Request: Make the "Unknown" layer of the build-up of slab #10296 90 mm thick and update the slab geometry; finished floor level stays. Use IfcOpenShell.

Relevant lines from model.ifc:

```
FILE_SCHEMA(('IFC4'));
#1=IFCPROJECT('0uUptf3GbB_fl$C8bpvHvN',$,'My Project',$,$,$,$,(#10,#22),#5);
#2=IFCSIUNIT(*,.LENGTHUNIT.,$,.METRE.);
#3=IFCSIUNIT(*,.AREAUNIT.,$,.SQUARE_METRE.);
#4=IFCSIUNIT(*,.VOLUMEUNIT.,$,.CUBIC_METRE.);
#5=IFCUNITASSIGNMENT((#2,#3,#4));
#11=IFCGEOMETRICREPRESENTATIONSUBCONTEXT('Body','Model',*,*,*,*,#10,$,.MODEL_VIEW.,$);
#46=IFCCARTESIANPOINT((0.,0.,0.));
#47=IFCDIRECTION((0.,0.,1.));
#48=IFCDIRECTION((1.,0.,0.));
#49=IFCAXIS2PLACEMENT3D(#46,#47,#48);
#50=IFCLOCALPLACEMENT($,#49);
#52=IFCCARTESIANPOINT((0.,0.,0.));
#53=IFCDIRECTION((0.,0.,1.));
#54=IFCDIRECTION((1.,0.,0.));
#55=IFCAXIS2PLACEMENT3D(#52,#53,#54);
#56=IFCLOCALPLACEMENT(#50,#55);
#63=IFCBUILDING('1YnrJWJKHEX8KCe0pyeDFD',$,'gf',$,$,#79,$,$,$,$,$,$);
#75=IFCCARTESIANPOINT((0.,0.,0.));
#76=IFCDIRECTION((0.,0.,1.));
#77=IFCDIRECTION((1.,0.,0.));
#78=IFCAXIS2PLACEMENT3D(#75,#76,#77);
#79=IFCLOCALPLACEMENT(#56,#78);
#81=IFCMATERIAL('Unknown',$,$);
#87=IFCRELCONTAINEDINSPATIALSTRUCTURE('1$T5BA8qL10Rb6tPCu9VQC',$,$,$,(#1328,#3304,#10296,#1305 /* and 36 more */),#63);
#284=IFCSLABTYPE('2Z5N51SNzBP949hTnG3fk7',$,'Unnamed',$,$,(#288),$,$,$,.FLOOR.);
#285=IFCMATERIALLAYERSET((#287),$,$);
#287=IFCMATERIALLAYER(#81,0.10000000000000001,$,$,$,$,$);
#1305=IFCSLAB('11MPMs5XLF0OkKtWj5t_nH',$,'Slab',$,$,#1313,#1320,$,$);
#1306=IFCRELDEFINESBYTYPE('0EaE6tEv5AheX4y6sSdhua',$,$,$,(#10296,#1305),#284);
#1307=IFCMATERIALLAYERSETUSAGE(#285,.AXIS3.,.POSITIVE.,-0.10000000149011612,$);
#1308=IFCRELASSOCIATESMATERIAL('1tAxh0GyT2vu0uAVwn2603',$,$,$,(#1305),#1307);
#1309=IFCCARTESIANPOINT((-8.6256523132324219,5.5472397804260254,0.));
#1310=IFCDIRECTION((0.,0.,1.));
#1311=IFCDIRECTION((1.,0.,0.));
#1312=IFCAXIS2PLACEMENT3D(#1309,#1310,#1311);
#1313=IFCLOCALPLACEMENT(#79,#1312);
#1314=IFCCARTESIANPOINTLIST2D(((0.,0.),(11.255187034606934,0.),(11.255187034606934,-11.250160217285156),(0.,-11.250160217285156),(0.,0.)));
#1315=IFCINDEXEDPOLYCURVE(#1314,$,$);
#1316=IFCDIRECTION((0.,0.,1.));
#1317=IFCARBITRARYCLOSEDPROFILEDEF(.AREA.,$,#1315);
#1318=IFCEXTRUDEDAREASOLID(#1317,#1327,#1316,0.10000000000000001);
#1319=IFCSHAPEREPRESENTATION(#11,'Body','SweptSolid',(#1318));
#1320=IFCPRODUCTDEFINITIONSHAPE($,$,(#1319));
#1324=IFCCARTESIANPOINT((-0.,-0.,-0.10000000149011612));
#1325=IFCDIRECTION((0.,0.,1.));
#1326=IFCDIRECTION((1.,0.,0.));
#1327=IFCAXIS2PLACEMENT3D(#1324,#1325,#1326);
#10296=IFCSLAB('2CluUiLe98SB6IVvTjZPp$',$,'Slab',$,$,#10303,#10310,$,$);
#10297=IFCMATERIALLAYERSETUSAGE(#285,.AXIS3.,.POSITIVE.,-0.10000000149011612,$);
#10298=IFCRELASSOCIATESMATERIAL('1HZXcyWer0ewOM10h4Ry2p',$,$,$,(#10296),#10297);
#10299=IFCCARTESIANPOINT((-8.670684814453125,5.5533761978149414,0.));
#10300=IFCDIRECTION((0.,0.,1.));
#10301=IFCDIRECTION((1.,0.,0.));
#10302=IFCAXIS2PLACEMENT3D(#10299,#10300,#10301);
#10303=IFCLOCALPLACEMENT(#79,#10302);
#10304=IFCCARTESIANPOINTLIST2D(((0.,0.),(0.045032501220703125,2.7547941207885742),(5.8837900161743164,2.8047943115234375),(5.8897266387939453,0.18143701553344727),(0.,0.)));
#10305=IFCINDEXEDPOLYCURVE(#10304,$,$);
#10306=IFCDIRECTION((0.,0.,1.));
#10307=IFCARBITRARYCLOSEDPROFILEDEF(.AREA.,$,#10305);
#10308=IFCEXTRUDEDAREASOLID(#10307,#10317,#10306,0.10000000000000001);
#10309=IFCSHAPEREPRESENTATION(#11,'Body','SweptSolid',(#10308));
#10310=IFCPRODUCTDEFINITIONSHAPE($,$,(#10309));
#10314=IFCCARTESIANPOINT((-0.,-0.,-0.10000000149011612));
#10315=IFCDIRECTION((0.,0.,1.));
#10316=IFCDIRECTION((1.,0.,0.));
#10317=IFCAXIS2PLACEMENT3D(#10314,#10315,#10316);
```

```python
import ifcopenshell
import ifcopenshell.util.element
import ifcopenshell.util.representation
import ifcopenshell.util.unit

model = ifcopenshell.open("model.ifc")
unit_scale = ifcopenshell.util.unit.calculate_unit_scale(model)

layer_set = model.by_id(285)
layer = next(l for l in layer_set.MaterialLayers if l.Material and l.Material.Name == "Unknown")
change = 0.09 / unit_scale - layer.LayerThickness
layer.LayerThickness += change

# The layer set is shared, so every slab that uses it gets the new thickness.
slabs = [e for e in ifcopenshell.util.element.get_elements_by_material(model, layer_set) if e.is_a("IfcSlab")]
for slab in sorted(slabs, key=lambda e: e.id()):
    body = ifcopenshell.util.representation.get_representation(slab, "Model", "Body")
    solid = body.Items[0]
    old_depth = solid.Depth
    solid.Depth += change
    # Extruded upwards: lower the start of the extrusion so the top stays.
    x, y, z = solid.Position.Location.Coordinates
    solid.Position.Location = model.createIfcCartesianPoint((x, y, z - change))
    print(slab.id(), f"{old_depth:g} -> {solid.Depth:g}")

# The layers are counted up from the underside, which has moved.
for usage in {ifcopenshell.util.element.get_material(slab) for slab in slabs}:
    usage.OffsetFromReferenceLine -= change

model.write("model_v2.ifc")
```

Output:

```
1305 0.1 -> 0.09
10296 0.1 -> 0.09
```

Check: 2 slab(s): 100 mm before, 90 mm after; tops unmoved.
